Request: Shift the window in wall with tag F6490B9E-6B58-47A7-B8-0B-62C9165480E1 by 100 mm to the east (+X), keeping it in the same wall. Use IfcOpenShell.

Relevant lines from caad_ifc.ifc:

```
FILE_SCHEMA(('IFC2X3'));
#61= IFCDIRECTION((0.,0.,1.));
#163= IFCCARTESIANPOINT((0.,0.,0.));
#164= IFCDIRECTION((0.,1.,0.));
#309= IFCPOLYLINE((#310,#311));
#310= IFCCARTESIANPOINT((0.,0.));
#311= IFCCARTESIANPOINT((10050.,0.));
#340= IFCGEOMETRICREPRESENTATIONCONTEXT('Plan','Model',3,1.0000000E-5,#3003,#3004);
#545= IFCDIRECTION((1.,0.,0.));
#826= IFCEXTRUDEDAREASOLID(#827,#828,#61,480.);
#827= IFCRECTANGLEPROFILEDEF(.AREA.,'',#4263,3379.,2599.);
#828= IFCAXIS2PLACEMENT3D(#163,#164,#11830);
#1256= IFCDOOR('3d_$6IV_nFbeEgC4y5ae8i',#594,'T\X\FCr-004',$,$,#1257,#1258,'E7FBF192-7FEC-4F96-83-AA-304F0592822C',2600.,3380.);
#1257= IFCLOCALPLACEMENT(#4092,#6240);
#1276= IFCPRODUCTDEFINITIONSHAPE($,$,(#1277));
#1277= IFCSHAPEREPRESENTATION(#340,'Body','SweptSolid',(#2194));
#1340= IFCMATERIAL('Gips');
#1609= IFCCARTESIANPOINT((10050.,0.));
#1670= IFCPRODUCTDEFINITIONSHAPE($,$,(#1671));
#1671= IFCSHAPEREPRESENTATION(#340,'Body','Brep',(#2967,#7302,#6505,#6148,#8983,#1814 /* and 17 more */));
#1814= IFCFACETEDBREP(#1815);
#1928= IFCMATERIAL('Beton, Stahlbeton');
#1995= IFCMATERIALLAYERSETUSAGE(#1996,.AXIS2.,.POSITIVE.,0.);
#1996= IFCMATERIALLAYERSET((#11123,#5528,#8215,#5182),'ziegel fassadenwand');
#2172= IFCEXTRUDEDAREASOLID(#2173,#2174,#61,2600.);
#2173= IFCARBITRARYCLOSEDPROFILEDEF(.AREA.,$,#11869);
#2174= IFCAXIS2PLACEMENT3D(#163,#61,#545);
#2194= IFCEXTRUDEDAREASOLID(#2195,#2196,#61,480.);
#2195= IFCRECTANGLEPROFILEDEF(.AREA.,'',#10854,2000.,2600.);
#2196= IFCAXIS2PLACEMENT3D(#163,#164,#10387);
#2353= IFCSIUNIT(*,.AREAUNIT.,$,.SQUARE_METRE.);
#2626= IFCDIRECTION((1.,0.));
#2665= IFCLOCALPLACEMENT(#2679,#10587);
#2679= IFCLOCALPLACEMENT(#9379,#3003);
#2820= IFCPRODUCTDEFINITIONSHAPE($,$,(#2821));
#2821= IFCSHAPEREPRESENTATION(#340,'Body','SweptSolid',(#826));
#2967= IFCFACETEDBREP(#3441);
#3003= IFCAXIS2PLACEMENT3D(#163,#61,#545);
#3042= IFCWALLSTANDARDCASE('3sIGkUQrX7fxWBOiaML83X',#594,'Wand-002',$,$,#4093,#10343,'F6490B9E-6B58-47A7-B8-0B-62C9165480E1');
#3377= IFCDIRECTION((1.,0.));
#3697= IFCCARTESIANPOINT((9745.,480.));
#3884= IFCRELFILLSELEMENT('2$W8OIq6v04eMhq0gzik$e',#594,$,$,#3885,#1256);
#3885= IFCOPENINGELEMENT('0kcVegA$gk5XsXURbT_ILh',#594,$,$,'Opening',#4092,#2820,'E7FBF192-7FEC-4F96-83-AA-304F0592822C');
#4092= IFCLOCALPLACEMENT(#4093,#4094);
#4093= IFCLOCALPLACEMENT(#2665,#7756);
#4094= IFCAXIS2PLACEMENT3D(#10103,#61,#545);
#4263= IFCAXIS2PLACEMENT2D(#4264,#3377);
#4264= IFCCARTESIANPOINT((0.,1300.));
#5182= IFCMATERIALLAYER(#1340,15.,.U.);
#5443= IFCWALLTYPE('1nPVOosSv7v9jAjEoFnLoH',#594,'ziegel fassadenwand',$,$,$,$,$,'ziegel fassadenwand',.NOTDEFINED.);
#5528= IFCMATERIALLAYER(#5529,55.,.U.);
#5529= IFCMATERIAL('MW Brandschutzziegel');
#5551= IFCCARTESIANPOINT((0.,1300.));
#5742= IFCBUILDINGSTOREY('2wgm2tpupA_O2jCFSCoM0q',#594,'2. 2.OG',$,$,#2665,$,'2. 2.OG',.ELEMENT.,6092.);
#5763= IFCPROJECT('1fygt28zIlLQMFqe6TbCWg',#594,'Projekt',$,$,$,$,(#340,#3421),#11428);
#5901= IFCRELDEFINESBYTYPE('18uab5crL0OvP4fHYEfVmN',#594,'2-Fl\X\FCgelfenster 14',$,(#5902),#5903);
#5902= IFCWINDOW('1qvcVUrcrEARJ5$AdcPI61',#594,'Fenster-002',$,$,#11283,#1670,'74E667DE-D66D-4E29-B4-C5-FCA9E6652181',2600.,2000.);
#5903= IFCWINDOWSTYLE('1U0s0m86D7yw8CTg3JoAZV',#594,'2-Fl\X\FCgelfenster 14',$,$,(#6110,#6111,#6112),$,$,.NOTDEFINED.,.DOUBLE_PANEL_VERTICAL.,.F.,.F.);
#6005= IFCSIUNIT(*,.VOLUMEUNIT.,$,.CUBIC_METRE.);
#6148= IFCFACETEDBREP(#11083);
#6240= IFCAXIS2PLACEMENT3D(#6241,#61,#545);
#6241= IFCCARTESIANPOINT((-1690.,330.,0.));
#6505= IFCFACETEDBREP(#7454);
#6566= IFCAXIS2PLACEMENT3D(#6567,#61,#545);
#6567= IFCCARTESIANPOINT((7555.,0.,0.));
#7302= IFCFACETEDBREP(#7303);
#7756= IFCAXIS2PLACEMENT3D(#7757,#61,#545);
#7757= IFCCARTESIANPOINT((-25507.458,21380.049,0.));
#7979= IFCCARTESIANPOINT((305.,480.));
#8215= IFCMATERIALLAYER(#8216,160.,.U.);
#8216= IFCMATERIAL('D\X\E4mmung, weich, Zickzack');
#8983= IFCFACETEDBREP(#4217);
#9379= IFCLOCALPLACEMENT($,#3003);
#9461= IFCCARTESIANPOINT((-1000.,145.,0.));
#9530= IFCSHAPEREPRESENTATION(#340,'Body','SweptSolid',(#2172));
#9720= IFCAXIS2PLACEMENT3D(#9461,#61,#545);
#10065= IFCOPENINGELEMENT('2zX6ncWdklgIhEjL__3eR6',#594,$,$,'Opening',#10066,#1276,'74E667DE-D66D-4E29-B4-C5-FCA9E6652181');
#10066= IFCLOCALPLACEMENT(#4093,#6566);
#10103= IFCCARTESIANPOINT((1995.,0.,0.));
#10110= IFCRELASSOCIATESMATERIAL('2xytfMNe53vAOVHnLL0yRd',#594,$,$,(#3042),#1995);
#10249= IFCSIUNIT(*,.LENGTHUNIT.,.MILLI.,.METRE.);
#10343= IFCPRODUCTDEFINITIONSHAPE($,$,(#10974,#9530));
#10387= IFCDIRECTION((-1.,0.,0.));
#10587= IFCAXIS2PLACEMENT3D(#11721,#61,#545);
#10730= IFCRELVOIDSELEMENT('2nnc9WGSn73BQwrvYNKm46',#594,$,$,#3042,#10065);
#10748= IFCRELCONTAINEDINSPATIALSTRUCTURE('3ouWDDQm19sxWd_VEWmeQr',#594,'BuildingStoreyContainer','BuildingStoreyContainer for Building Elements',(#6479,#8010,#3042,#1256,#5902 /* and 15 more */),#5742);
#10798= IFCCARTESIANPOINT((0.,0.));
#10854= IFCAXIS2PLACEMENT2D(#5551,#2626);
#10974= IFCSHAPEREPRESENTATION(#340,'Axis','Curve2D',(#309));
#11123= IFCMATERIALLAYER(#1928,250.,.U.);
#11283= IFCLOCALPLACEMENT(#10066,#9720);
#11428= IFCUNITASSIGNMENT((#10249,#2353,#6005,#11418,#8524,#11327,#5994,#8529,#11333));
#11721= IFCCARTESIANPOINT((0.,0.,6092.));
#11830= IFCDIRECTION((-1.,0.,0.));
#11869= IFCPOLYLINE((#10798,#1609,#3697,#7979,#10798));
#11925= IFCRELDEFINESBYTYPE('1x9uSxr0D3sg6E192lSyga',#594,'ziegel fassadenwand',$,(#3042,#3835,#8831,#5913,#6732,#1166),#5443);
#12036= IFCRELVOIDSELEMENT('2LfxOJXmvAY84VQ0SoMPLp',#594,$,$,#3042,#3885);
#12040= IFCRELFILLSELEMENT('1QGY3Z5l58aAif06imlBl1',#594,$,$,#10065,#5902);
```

```python
import ifcopenshell
import ifcopenshell.api.geometry
import ifcopenshell.util.placement
import ifcopenshell.util.unit

model = ifcopenshell.open("caad_ifc.ifc")
unit_scale = ifcopenshell.util.unit.calculate_unit_scale(model)

window = model.by_guid("1qvcVUrcrEARJ5$AdcPI61")
opening = window.FillsVoids[0].RelatingOpeningElement
wall = opening.VoidsElements[0].RelatingBuildingElement

wall_matrix = ifcopenshell.util.placement.get_local_placement(wall.ObjectPlacement)
shift = wall_matrix[:3, 0] * 0.1 / unit_scale
before = ifcopenshell.util.placement.get_local_placement(window.ObjectPlacement)[:3, 3].copy()

# The window is placed relative to its opening, so it follows when the opening moves.
matrix = ifcopenshell.util.placement.get_local_placement(opening.ObjectPlacement)
matrix[:3, 3] += shift
ifcopenshell.api.geometry.edit_object_placement(
    model, product=opening, matrix=matrix, is_si=False, should_transform_children=True
)

after = ifcopenshell.util.placement.get_local_placement(window.ObjectPlacement)[:3, 3]
print("window moved by", (after - before).round(3) + 0.0)

model.write("caad_ifc_updated.ifc")
```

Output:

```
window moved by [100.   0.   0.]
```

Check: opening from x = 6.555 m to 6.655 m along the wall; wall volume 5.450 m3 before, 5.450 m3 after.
